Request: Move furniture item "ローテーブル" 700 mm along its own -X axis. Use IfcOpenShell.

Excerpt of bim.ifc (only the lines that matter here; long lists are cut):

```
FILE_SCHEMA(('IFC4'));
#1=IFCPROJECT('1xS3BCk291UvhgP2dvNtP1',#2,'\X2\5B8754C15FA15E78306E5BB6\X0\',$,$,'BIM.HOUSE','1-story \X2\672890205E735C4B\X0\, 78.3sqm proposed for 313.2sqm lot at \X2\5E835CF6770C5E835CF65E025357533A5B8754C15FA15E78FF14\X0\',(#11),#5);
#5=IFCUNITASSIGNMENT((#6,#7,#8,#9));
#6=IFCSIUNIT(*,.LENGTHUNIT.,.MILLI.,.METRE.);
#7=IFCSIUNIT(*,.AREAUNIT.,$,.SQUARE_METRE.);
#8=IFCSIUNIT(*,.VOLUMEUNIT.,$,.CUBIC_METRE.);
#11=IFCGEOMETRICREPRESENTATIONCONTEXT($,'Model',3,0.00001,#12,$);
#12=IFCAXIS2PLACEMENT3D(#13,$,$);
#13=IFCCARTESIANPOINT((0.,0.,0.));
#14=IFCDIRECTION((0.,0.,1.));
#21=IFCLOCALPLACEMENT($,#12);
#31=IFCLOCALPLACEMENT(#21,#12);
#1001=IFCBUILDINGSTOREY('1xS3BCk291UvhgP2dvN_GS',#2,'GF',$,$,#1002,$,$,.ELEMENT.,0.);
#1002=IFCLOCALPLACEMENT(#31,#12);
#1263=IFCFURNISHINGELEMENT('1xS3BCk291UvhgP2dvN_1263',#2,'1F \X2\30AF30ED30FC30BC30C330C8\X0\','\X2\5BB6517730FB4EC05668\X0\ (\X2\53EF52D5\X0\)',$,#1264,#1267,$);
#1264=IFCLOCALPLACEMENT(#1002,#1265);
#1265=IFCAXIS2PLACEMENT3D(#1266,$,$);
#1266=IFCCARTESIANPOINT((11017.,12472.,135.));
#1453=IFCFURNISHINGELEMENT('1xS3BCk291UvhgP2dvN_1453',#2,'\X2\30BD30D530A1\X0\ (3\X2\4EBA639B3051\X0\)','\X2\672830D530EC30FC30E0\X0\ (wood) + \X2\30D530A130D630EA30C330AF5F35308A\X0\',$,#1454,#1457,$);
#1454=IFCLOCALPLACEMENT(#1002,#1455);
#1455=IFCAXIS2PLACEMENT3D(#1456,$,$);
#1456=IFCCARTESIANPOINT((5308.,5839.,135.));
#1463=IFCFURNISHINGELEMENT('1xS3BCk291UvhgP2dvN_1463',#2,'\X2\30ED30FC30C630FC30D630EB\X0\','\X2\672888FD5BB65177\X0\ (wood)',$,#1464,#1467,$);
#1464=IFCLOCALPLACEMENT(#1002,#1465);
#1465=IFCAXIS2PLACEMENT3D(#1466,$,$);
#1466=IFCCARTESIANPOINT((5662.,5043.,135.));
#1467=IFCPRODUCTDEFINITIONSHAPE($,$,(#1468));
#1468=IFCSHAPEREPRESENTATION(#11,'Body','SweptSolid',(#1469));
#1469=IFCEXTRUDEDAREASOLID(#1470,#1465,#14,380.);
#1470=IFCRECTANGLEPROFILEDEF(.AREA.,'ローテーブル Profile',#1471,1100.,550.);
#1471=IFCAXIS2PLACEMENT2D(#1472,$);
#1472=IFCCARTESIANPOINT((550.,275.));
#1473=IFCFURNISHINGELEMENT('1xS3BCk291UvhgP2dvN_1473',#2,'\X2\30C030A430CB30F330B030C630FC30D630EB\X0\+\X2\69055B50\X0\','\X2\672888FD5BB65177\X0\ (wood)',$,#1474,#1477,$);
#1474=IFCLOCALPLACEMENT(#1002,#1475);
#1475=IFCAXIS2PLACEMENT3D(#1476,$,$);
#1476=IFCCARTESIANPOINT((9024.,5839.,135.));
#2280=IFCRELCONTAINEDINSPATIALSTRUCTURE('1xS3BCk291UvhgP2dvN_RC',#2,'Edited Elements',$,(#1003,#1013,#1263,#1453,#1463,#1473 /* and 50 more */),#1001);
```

```python
import ifcopenshell
import ifcopenshell.api.geometry
import ifcopenshell.util.placement
import ifcopenshell.util.unit

model = ifcopenshell.open("bim.ifc")
unit_scale = ifcopenshell.util.unit.calculate_unit_scale(model)

item = model.by_guid("1xS3BCk291UvhgP2dvN_1463")
matrix = ifcopenshell.util.placement.get_local_placement(item.ObjectPlacement)
matrix[:3, 3] -= matrix[:3, 0] * 0.7 / unit_scale
ifcopenshell.api.geometry.edit_object_placement(model, product=item, matrix=matrix, is_si=False)

print(ifcopenshell.util.placement.get_local_placement(item.ObjectPlacement).round(3) + 0.0)

model.write("bim_updated.ifc")
```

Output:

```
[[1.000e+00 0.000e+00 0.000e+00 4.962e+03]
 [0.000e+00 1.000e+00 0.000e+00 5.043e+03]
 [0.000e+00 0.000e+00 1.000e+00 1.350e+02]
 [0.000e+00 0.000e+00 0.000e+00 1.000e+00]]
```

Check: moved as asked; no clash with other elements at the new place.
